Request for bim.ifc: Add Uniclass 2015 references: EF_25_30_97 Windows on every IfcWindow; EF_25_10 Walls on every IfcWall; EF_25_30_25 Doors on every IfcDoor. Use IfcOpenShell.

First a look at what the model holds.

```python
import ifcopenshell

model = ifcopenshell.open("bim.ifc")
print(model.schema)
print("classifications:", [c.Name for c in model.by_type("IfcClassification")])
for ifc_class in ("IfcDoor", "IfcRoof", "IfcStair", "IfcWall", "IfcWindow"):
    print(ifc_class, len(model.by_type(ifc_class)))
```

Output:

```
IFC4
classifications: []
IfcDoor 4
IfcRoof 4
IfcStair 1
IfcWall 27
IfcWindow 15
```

```python
import ifcopenshell
import ifcopenshell.api.classification

model = ifcopenshell.open("bim.ifc")

system = ifcopenshell.api.classification.add_classification(model, classification="Uniclass 2015")

codes = {
    "IfcWindow": ("EF_25_30_97", "Windows"),
    "IfcWall": ("EF_25_10", "Walls"),
    "IfcDoor": ("EF_25_30_25", "Doors"),
}
for ifc_class, (code, name) in codes.items():
    products = model.by_type(ifc_class)
    ifcopenshell.api.classification.add_reference(
        model, products=products, classification=system, identification=code, name=name
    )
    print(code, len(products))

model.write("bim-out.ifc")
```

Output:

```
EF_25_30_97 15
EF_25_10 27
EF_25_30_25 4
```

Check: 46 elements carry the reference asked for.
